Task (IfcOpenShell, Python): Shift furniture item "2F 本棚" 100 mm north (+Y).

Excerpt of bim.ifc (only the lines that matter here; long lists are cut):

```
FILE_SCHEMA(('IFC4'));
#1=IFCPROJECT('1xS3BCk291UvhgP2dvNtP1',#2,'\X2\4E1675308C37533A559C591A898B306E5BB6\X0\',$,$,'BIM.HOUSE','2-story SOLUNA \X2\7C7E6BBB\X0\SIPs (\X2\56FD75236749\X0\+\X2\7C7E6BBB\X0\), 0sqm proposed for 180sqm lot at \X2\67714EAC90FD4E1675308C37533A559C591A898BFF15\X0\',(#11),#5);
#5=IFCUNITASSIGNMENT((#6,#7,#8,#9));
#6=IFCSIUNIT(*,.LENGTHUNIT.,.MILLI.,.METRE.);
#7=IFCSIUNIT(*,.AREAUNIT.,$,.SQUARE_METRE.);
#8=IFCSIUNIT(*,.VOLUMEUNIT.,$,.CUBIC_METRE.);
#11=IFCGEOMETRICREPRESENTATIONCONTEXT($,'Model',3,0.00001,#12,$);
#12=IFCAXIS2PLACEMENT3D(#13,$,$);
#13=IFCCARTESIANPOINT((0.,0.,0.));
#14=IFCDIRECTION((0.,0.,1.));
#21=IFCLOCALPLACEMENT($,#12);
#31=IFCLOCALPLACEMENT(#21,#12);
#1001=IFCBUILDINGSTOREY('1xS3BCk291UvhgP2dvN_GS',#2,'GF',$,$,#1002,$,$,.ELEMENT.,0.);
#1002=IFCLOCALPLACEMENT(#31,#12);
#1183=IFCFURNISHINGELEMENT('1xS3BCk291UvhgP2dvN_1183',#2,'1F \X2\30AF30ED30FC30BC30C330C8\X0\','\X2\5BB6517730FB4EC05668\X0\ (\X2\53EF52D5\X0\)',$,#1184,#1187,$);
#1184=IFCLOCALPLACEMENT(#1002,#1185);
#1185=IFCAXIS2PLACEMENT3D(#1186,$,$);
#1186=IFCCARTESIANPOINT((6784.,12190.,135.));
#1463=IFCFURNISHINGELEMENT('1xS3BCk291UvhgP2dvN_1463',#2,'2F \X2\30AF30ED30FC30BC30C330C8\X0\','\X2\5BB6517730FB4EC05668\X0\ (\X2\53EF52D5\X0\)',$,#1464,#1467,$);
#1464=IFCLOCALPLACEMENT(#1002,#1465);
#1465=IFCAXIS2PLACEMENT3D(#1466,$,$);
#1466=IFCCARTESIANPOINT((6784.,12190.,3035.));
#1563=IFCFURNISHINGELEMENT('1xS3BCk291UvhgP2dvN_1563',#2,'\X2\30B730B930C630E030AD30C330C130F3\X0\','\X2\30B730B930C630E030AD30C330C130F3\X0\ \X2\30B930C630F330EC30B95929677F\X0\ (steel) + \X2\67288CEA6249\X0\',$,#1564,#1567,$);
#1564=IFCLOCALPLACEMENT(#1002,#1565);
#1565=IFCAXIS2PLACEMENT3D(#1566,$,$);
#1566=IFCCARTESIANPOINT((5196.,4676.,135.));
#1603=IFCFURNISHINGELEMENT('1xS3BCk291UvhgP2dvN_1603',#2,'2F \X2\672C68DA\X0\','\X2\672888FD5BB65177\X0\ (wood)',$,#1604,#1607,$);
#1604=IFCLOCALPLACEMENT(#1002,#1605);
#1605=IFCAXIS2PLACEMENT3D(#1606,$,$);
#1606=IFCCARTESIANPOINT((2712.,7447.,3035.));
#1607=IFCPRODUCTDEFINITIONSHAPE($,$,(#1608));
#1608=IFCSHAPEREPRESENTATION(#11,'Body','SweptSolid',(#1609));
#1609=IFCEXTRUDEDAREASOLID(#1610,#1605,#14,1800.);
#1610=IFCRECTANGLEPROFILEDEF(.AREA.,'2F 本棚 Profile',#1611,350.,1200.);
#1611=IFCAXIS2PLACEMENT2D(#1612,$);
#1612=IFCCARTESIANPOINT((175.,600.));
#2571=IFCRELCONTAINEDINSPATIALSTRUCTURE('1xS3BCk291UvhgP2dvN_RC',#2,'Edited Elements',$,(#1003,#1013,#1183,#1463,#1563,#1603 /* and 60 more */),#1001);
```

```python
import ifcopenshell
import ifcopenshell.api.geometry
import ifcopenshell.util.placement
import ifcopenshell.util.unit

model = ifcopenshell.open("bim.ifc")
unit_scale = ifcopenshell.util.unit.calculate_unit_scale(model)

item = model.by_guid("1xS3BCk291UvhgP2dvN_1603")
matrix = ifcopenshell.util.placement.get_local_placement(item.ObjectPlacement)
matrix[1, 3] += 0.1 / unit_scale
ifcopenshell.api.geometry.edit_object_placement(model, product=item, matrix=matrix, is_si=False)

print(ifcopenshell.util.placement.get_local_placement(item.ObjectPlacement).round(3) + 0.0)

model.write("bim_rev.ifc")
```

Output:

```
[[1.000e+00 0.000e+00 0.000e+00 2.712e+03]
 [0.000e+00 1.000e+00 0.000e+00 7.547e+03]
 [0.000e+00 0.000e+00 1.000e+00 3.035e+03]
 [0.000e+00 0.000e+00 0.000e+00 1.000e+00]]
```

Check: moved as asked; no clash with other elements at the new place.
